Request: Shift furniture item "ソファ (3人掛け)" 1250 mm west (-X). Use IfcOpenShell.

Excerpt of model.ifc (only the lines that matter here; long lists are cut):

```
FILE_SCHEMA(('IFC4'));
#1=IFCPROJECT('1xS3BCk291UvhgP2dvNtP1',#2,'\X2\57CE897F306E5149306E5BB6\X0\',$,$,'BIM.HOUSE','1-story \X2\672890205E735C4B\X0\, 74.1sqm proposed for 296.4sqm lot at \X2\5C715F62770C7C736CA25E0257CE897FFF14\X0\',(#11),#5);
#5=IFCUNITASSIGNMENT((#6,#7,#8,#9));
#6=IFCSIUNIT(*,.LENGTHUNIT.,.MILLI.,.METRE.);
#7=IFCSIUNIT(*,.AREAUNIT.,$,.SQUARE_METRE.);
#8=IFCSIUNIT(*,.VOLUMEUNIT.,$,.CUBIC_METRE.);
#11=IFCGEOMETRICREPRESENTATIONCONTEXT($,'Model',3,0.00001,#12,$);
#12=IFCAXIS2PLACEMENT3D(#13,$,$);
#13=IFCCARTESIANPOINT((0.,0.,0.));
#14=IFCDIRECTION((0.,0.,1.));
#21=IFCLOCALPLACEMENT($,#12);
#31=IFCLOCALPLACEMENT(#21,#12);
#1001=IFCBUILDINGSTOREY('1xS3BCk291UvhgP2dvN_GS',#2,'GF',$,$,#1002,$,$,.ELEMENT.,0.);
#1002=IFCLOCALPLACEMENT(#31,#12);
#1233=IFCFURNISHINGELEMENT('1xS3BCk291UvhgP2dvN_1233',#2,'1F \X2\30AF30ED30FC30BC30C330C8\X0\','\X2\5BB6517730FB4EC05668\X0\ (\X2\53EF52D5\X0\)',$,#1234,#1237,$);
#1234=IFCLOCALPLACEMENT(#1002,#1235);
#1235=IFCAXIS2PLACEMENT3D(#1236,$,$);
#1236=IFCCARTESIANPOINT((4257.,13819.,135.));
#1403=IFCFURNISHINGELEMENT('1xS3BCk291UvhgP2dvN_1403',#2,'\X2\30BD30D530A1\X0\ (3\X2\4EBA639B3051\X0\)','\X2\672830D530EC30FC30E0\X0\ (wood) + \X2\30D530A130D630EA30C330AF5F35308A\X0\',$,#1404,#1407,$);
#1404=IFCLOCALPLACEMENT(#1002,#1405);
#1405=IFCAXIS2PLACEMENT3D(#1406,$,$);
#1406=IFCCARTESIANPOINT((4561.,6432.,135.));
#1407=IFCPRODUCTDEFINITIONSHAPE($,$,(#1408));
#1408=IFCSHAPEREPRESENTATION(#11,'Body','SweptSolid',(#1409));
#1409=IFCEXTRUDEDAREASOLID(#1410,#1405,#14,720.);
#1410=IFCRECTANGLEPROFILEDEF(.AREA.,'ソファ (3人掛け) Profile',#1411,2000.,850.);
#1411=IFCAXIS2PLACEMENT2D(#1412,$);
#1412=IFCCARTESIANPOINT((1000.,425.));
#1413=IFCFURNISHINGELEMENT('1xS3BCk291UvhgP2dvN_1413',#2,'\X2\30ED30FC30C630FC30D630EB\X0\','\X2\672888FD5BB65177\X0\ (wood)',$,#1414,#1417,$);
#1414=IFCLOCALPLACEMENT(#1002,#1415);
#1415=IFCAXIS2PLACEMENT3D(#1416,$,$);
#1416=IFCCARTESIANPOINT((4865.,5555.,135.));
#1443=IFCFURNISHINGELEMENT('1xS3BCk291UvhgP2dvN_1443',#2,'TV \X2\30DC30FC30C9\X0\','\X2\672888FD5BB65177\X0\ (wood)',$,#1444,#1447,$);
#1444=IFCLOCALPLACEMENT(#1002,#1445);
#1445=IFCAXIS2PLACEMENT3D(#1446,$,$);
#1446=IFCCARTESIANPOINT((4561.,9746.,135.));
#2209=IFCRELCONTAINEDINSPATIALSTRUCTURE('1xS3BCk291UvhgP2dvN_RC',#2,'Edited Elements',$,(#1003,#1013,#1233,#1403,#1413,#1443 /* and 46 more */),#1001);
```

```python
import ifcopenshell
import ifcopenshell.api.geometry
import ifcopenshell.util.placement
import ifcopenshell.util.unit

model = ifcopenshell.open("model.ifc")
unit_scale = ifcopenshell.util.unit.calculate_unit_scale(model)

item = model.by_guid("1xS3BCk291UvhgP2dvN_1403")
matrix = ifcopenshell.util.placement.get_local_placement(item.ObjectPlacement)
matrix[0, 3] -= 1.25 / unit_scale
ifcopenshell.api.geometry.edit_object_placement(model, product=item, matrix=matrix, is_si=False)

print(ifcopenshell.util.placement.get_local_placement(item.ObjectPlacement).round(3) + 0.0)

model.write("model-out.ifc")
```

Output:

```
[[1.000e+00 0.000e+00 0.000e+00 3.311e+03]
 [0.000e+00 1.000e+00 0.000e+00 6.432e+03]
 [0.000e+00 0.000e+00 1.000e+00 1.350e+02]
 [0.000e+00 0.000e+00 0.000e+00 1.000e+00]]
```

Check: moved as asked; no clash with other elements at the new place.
